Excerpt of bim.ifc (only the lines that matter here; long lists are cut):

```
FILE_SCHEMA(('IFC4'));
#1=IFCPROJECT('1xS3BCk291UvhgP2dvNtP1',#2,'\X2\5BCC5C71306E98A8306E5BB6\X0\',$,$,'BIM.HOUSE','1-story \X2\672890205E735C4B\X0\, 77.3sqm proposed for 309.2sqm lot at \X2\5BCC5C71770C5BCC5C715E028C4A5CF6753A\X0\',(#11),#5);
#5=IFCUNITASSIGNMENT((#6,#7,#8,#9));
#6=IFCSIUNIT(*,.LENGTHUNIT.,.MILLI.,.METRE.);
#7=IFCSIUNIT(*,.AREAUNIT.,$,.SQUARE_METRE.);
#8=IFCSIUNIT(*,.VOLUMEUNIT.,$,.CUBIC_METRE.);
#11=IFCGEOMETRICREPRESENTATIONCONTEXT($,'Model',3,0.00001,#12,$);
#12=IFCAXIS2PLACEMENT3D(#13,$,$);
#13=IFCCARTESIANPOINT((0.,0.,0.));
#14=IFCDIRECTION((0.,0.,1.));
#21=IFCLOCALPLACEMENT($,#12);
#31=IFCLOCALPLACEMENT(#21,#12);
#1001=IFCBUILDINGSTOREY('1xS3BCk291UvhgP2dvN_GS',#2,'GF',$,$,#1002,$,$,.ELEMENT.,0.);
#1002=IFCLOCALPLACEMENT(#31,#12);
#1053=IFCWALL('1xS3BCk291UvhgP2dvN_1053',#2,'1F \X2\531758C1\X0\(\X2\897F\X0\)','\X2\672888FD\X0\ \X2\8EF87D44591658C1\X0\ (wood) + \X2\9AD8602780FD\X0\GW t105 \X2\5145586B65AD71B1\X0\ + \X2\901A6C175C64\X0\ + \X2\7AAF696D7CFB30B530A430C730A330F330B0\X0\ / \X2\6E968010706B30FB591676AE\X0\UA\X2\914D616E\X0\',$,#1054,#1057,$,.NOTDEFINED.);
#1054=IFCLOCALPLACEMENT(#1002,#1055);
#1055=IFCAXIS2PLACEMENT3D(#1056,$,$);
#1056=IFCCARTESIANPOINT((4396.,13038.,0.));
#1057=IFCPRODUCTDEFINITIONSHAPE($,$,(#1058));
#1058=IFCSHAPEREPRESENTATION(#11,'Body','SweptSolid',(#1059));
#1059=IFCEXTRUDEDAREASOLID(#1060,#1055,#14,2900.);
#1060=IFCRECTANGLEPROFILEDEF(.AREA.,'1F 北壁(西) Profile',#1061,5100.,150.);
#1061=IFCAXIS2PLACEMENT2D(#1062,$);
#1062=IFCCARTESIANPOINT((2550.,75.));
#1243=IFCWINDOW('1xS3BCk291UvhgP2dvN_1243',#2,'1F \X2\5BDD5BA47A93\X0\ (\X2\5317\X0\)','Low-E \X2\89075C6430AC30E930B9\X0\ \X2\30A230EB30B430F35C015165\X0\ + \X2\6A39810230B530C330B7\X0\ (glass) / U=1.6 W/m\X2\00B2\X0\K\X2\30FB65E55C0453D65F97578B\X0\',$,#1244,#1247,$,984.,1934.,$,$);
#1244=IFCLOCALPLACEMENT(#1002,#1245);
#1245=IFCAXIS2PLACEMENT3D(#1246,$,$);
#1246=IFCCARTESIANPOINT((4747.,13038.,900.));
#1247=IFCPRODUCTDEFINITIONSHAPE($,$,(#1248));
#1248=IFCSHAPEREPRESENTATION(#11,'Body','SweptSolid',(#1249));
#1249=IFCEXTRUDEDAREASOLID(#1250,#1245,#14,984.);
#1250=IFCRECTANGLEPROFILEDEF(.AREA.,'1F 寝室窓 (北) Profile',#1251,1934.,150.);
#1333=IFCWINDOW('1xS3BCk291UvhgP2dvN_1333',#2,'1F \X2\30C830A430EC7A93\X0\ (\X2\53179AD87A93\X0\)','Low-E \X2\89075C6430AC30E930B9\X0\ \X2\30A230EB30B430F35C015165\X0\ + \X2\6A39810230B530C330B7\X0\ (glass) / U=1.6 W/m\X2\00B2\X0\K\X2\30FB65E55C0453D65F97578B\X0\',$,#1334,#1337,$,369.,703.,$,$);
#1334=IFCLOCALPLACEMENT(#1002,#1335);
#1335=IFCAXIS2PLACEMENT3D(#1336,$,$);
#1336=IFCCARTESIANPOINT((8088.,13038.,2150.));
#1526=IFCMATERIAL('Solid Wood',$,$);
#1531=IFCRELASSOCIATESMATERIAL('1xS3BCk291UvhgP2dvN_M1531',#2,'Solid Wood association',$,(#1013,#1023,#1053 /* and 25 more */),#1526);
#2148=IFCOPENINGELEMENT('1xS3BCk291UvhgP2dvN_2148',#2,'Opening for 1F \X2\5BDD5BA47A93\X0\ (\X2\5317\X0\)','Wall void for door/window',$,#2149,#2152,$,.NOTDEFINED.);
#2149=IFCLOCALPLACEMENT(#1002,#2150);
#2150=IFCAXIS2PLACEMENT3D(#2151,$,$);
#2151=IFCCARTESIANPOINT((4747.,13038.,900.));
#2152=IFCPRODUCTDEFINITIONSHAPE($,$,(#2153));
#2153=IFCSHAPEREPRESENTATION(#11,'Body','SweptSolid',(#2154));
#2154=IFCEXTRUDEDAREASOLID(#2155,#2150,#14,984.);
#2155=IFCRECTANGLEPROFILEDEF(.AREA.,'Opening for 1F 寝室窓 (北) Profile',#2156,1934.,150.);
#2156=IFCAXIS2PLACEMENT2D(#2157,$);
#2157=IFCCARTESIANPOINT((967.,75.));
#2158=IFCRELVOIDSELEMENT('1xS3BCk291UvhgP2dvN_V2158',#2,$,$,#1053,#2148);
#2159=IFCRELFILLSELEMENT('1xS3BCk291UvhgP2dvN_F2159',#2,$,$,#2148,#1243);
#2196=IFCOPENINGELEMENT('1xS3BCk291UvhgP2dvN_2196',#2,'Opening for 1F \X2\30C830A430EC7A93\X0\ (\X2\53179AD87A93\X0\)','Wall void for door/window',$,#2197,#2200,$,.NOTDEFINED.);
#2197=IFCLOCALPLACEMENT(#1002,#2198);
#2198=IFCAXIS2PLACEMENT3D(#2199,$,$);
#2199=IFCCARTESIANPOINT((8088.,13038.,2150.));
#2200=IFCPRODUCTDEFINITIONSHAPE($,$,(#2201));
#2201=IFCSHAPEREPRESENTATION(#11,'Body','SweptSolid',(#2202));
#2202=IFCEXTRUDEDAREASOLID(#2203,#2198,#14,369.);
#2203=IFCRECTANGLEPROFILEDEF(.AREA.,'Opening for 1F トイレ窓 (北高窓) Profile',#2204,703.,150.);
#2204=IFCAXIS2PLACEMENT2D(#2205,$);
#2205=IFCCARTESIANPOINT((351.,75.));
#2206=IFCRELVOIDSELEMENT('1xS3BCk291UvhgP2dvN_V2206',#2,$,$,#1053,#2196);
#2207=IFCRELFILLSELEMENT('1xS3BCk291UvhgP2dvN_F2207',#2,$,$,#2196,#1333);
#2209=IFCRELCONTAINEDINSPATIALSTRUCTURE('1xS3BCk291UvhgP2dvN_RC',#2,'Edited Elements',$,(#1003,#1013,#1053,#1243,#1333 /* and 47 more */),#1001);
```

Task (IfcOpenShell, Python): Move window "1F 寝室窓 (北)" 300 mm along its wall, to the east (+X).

```python
import ifcopenshell
import ifcopenshell.api.geometry
import ifcopenshell.util.placement
import ifcopenshell.util.unit

model = ifcopenshell.open("bim.ifc")
unit_scale = ifcopenshell.util.unit.calculate_unit_scale(model)

window = model.by_id(1243)
opening = window.FillsVoids[0].RelatingOpeningElement
wall = opening.VoidsElements[0].RelatingBuildingElement

wall_matrix = ifcopenshell.util.placement.get_local_placement(wall.ObjectPlacement)
shift = wall_matrix[:3, 0] * 0.3 / unit_scale
before = ifcopenshell.util.placement.get_local_placement(window.ObjectPlacement)[:3, 3].copy()

# The window is not placed relative to its opening, so move both.
for product in (opening, window):
    matrix = ifcopenshell.util.placement.get_local_placement(product.ObjectPlacement)
    matrix[:3, 3] += shift
    ifcopenshell.api.geometry.edit_object_placement(model, product=product, matrix=matrix, is_si=False)

after = ifcopenshell.util.placement.get_local_placement(window.ObjectPlacement)[:3, 3]
print("window moved by", (after - before).round(3) + 0.0)

model.write("bim_updated.ifc")
```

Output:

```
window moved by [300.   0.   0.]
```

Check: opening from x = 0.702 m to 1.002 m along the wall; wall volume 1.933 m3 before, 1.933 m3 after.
